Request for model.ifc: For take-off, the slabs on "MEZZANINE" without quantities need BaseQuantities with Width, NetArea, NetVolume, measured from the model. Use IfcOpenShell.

First a look at what the model holds.

```python
import ifcopenshell
import ifcopenshell.util.element
import ifcopenshell.util.unit

model = ifcopenshell.open("model.ifc")
print(model.schema)
for unit_type in ("LENGTHUNIT", "AREAUNIT", "VOLUMEUNIT"):
    print(unit_type, ifcopenshell.util.unit.calculate_unit_scale(model, unit_type))
storey = next(s for s in model.by_type("IfcBuildingStorey") if s.Name == "MEZZANINE")
slabs = [e for e in ifcopenshell.util.element.get_decomposition(storey) if e.is_a("IfcSlab")]
for e in sorted(slabs, key=lambda e: e.id()):
    print(e.id(), e.is_a(), e.Name, list(ifcopenshell.util.element.get_psets(e, qtos_only=True)), sep=" | ")
```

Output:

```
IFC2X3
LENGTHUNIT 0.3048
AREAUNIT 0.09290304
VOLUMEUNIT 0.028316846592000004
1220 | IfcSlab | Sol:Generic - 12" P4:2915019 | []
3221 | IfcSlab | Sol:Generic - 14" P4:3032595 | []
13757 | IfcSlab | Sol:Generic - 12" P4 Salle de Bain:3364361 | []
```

```python
import ifcopenshell
import ifcopenshell.api.pset
import ifcopenshell.geom
import ifcopenshell.util.element
import ifcopenshell.util.shape
import ifcopenshell.util.unit

model = ifcopenshell.open("model.ifc")
unit_scale = ifcopenshell.util.unit.calculate_unit_scale(model)
area_scale = ifcopenshell.util.unit.calculate_unit_scale(model, "AREAUNIT")
volume_scale = ifcopenshell.util.unit.calculate_unit_scale(model, "VOLUMEUNIT")
settings = ifcopenshell.geom.settings()

storey = next(s for s in model.by_type("IfcBuildingStorey") if s.Name == "MEZZANINE")
slabs = [e for e in ifcopenshell.util.element.get_decomposition(storey) if e.is_a("IfcSlab")]

for e in sorted(slabs, key=lambda e: e.id()):
    if ifcopenshell.util.element.get_psets(e, qtos_only=True, should_inherit=False):
        continue
    # Geometry comes back in metres, in the element's own axes.
    shape = ifcopenshell.geom.create_shape(settings, e)
    values = {
        "Width": ifcopenshell.util.shape.get_z(shape.geometry) / unit_scale,
        "NetArea": ifcopenshell.util.shape.get_footprint_area(shape.geometry) / area_scale,
        "NetVolume": ifcopenshell.util.shape.get_volume(shape.geometry) / volume_scale,
    }
    qto = ifcopenshell.api.pset.add_qto(model, product=e, name="BaseQuantities")
    ifcopenshell.api.pset.edit_qto(model, qto=qto, properties=values)
    print(e.id(), {k: round(v, 3) for k, v in values.items()})

model.write("model-out.ifc")
```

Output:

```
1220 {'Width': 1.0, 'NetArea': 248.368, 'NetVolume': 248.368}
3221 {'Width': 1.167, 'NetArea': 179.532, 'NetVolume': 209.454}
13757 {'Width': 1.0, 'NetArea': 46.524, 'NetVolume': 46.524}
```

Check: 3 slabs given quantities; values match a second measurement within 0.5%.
